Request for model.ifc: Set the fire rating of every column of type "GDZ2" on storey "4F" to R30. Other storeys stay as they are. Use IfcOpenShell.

First a look at what the model holds.

```python
import ifcopenshell
import ifcopenshell.util.element

model = ifcopenshell.open("model.ifc")
print(model.schema)
storey = next(s for s in model.by_type("IfcBuildingStorey") if s.Name == "4F")
columns = [e for e in ifcopenshell.util.element.get_decomposition(storey) if e.is_a("IfcColumn")]
seen = {}
for e in columns:
    element_type = ifcopenshell.util.element.get_type(e)
    key = (element_type.Name if element_type != e and element_type else None, ifcopenshell.util.element.get_pset(e, "Pset_ColumnCommon", "FireRating"))
    seen[key] = seen.get(key, 0) + 1
for (name, value), count in sorted(seen.items(), key=str):
    print(count, "x", name, "|", value)
```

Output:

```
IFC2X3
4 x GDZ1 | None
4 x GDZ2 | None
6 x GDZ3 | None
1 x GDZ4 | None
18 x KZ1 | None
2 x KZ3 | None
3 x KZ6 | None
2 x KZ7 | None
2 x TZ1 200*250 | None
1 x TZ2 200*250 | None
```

```python
import ifcopenshell
import ifcopenshell.api.pset
import ifcopenshell.util.element

model = ifcopenshell.open("model.ifc")

storey = next(s for s in model.by_type("IfcBuildingStorey") if s.Name == "4F")
columns = [e for e in ifcopenshell.util.element.get_decomposition(storey) if e.is_a("IfcColumn")]

count = 0
for e in columns:
    element_type = ifcopenshell.util.element.get_type(e)
    if element_type in (None, e) or element_type.Name != "GDZ2":
        continue
    # add_pset returns the element's existing set when there is one.
    pset = ifcopenshell.api.pset.add_pset(model, product=e, name="Pset_ColumnCommon")
    ifcopenshell.api.pset.edit_pset(model, pset=pset, properties={"FireRating": "R30"})
    count += 1

print(count, "columns updated")

model.write("model_v2.ifc")
```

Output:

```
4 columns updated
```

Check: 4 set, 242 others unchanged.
